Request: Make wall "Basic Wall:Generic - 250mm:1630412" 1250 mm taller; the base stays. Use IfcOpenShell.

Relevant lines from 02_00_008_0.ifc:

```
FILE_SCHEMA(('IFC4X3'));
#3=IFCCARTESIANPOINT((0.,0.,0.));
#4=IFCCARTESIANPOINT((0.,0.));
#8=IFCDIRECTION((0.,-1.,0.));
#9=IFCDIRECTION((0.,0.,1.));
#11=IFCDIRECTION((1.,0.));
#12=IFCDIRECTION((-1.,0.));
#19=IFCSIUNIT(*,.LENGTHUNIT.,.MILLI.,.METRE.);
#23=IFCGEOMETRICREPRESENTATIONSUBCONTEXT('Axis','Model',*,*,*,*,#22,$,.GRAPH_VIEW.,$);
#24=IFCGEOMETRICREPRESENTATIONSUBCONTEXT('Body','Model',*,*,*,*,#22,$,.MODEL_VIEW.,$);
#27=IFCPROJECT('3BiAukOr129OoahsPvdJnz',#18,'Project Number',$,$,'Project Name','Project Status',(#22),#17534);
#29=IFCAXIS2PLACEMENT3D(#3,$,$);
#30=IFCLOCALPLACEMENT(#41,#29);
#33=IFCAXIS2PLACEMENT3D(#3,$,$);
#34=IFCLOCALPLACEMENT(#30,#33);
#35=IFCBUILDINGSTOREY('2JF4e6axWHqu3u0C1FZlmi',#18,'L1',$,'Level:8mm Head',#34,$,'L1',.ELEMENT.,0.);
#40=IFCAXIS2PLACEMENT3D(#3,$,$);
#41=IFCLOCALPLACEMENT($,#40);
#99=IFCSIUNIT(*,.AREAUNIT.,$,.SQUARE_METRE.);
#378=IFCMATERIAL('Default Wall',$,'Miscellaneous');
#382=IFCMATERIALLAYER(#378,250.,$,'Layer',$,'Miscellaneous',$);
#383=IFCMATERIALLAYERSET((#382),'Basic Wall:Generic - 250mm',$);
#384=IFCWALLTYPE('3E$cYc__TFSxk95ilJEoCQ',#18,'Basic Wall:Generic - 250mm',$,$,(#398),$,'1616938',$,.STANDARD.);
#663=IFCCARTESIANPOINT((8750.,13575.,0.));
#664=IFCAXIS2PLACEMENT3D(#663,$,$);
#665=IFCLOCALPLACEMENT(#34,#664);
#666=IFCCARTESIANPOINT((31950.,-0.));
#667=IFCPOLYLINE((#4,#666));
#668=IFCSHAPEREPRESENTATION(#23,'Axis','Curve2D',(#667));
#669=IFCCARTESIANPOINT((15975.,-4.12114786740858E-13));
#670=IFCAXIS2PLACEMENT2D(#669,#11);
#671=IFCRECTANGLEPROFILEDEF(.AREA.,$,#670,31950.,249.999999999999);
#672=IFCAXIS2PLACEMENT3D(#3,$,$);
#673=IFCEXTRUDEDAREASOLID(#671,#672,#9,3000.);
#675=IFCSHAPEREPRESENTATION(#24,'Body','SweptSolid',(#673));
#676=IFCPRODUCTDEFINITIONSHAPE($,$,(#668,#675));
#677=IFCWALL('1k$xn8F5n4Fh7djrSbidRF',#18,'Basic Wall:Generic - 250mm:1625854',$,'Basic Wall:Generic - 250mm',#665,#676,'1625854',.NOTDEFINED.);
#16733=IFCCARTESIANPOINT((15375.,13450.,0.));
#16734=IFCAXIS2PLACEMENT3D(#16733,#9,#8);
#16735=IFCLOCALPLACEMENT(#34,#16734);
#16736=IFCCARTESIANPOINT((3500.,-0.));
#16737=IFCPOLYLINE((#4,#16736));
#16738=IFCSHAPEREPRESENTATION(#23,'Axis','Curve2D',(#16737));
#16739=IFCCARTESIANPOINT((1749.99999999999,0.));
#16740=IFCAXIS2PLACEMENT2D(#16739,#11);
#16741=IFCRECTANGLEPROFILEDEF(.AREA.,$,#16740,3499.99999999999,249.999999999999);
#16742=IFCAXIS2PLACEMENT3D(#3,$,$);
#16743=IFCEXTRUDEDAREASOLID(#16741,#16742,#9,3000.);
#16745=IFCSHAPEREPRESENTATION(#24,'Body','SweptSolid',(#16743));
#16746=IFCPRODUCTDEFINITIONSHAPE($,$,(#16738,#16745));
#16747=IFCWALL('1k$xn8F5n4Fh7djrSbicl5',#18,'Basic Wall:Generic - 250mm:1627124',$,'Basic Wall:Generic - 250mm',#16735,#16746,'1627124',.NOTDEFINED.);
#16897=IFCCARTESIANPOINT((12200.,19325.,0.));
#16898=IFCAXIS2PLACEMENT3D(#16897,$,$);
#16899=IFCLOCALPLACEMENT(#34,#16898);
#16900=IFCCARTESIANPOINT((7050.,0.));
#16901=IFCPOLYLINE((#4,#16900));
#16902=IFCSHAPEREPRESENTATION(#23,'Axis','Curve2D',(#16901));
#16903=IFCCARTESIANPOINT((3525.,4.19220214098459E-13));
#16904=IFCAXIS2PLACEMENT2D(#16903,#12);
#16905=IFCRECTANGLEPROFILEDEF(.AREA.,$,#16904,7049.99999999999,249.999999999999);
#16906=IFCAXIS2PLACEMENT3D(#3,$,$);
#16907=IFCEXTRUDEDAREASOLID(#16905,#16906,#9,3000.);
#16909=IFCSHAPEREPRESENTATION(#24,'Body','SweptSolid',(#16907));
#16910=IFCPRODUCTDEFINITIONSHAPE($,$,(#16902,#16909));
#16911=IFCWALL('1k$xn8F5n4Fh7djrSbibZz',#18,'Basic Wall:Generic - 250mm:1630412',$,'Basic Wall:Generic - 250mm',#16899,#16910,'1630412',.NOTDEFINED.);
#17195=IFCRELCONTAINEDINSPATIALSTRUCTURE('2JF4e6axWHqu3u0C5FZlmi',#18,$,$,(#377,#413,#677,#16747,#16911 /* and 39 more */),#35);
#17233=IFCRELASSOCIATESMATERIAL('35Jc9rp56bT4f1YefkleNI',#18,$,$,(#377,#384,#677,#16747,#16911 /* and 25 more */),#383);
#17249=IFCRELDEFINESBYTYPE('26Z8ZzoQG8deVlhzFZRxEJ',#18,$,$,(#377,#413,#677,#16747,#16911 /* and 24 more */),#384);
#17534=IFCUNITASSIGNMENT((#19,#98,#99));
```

```python
import ifcopenshell
import ifcopenshell.geom
import ifcopenshell.util.representation
import ifcopenshell.util.shape
import ifcopenshell.util.unit

model = ifcopenshell.open("02_00_008_0.ifc")
unit_scale = ifcopenshell.util.unit.calculate_unit_scale(model)
settings = ifcopenshell.geom.settings()


def volume(element):
    """Net volume in cubic metres, openings subtracted."""
    shape = ifcopenshell.geom.create_shape(settings, element)
    return ifcopenshell.util.shape.get_volume(shape.geometry)


wall = model.by_guid("1k$xn8F5n4Fh7djrSbibZz")
before = volume(wall)

body = ifcopenshell.util.representation.get_representation(wall, "Model", "Body")
solid = body.Items[0]
old_height = solid.Depth
solid.Depth += 1.25 / unit_scale
after = volume(wall)

print(f"height {old_height:g} -> {solid.Depth:g}, volume {before:.3f} -> {after:.3f} m3")

model.write("02_00_008_0_rev.ifc")
```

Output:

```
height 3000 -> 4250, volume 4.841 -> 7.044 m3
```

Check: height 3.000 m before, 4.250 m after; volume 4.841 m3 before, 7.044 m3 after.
